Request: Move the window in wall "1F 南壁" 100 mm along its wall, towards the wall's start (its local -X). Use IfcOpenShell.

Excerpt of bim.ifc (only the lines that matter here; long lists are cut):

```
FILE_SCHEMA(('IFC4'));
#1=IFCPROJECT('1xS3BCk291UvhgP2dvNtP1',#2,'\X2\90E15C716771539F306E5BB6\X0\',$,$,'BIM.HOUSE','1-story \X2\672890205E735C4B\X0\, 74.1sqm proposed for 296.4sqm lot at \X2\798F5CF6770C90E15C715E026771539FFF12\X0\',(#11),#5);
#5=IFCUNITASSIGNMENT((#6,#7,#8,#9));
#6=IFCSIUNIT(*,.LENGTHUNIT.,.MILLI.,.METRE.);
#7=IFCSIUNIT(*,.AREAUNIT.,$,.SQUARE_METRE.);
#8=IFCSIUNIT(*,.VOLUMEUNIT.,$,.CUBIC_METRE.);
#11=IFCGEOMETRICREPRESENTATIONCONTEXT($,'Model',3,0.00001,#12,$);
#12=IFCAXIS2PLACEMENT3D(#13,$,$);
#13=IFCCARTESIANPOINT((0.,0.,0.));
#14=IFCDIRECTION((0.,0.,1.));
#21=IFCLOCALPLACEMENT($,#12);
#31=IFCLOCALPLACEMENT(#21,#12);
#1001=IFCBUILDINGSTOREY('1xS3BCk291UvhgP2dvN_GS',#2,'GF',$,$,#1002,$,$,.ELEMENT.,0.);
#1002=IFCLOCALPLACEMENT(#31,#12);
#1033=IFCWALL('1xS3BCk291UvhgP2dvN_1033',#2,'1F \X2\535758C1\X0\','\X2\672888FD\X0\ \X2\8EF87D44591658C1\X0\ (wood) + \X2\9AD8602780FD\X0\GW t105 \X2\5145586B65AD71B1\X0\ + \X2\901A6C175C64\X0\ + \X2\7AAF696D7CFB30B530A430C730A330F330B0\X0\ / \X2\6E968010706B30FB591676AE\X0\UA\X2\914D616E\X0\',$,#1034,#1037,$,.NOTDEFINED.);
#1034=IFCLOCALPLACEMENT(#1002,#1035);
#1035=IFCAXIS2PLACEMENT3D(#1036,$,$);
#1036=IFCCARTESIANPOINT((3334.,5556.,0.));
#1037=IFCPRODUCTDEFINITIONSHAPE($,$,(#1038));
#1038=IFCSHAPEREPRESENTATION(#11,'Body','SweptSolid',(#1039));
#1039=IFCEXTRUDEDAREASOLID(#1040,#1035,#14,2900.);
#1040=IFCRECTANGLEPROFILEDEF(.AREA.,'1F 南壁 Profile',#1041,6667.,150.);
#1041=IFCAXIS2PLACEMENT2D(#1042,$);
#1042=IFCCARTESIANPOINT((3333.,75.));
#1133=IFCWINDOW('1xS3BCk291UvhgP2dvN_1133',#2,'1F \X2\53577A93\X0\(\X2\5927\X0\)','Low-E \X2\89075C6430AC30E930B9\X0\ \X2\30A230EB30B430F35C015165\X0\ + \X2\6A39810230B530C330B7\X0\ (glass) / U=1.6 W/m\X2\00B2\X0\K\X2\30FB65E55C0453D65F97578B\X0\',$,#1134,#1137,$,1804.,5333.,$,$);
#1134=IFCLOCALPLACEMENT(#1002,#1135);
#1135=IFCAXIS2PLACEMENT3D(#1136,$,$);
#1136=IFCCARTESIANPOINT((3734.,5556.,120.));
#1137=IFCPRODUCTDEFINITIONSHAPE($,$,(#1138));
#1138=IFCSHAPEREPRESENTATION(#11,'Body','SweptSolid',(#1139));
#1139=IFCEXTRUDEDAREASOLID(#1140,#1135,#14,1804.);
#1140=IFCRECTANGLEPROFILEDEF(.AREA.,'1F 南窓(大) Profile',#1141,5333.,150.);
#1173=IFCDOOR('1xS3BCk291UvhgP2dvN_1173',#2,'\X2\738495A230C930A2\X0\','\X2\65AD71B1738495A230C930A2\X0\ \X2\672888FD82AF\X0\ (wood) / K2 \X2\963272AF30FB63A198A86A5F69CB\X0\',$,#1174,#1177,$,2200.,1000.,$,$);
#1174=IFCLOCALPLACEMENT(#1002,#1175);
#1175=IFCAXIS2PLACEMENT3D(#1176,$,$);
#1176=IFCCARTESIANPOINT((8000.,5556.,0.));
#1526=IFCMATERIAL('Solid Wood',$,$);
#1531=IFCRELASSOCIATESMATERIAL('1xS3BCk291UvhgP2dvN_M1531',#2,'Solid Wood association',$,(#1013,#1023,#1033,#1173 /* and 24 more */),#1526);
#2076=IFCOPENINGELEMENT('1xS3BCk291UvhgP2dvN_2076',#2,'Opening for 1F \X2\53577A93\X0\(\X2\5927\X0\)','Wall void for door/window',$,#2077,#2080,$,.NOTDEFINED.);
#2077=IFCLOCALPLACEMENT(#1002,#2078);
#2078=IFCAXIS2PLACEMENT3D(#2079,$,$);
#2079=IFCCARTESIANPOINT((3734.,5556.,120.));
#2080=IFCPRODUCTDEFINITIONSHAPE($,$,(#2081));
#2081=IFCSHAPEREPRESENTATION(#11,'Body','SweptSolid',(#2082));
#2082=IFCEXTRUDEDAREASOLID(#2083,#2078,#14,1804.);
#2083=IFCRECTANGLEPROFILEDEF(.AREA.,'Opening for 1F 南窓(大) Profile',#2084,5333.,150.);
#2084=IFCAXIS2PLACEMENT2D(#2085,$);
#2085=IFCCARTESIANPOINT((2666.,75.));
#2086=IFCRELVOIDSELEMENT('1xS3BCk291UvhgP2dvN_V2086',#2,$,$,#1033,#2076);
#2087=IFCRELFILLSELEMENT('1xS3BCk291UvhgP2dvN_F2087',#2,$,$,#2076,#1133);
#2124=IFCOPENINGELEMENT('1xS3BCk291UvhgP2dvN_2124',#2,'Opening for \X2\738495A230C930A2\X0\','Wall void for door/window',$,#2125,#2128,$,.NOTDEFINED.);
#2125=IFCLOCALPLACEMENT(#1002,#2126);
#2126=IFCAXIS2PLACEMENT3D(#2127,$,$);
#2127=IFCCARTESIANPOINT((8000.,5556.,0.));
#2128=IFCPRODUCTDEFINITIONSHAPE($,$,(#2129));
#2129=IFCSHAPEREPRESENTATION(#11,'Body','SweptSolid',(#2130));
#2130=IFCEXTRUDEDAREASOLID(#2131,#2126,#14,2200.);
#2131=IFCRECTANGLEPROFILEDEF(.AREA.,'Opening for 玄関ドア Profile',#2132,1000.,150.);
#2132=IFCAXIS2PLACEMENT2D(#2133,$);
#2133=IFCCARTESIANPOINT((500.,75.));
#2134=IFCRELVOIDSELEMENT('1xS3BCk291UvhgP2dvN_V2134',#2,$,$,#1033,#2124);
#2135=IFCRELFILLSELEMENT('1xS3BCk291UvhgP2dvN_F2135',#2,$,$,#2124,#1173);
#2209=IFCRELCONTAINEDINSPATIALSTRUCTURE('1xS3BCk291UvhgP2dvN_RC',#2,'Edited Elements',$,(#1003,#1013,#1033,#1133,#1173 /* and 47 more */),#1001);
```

```python
import ifcopenshell
import ifcopenshell.api.geometry
import ifcopenshell.util.placement
import ifcopenshell.util.unit

model = ifcopenshell.open("bim.ifc")
unit_scale = ifcopenshell.util.unit.calculate_unit_scale(model)

window = model.by_id(1133)
opening = window.FillsVoids[0].RelatingOpeningElement
wall = opening.VoidsElements[0].RelatingBuildingElement

wall_matrix = ifcopenshell.util.placement.get_local_placement(wall.ObjectPlacement)
shift = wall_matrix[:3, 0] * -0.1 / unit_scale
before = ifcopenshell.util.placement.get_local_placement(window.ObjectPlacement)[:3, 3].copy()

# The window is not placed relative to its opening, so move both.
for product in (opening, window):
    matrix = ifcopenshell.util.placement.get_local_placement(product.ObjectPlacement)
    matrix[:3, 3] += shift
    ifcopenshell.api.geometry.edit_object_placement(model, product=product, matrix=matrix, is_si=False)

after = ifcopenshell.util.placement.get_local_placement(window.ObjectPlacement)[:3, 3]
print("window moved by", (after - before).round(3) + 0.0)

model.write("bim_v2.ifc")
```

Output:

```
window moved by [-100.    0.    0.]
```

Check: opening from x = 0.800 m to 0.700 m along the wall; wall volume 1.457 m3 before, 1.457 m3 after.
